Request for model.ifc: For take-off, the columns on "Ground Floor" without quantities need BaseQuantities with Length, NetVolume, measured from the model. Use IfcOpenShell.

First a look at what the model holds.

```python
import ifcopenshell
import ifcopenshell.util.element
import ifcopenshell.util.unit

model = ifcopenshell.open("model.ifc")
print(model.schema)
for unit_type in ("LENGTHUNIT", "AREAUNIT", "VOLUMEUNIT"):
    print(unit_type, ifcopenshell.util.unit.calculate_unit_scale(model, unit_type))
storey = next(s for s in model.by_type("IfcBuildingStorey") if s.Name == "Ground Floor")
columns = [e for e in ifcopenshell.util.element.get_decomposition(storey) if e.is_a("IfcColumn")]
for e in sorted(columns, key=lambda e: e.id()):
    print(e.id(), e.is_a(), e.Name, list(ifcopenshell.util.element.get_psets(e, qtos_only=True)), sep=" | ")
```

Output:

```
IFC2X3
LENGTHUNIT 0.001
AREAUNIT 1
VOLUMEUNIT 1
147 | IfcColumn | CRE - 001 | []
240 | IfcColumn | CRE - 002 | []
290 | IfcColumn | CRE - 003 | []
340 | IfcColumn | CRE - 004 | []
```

```python
import ifcopenshell
import ifcopenshell.api.pset
import ifcopenshell.geom
import ifcopenshell.util.element
import ifcopenshell.util.shape
import ifcopenshell.util.unit

model = ifcopenshell.open("model.ifc")
unit_scale = ifcopenshell.util.unit.calculate_unit_scale(model)
volume_scale = ifcopenshell.util.unit.calculate_unit_scale(model, "VOLUMEUNIT")
settings = ifcopenshell.geom.settings()

storey = next(s for s in model.by_type("IfcBuildingStorey") if s.Name == "Ground Floor")
columns = [e for e in ifcopenshell.util.element.get_decomposition(storey) if e.is_a("IfcColumn")]

for e in sorted(columns, key=lambda e: e.id()):
    if ifcopenshell.util.element.get_psets(e, qtos_only=True, should_inherit=False):
        continue
    # Geometry comes back in metres, in the element's own axes.
    shape = ifcopenshell.geom.create_shape(settings, e)
    values = {
        "Length": ifcopenshell.util.shape.get_z(shape.geometry) / unit_scale,
        "NetVolume": ifcopenshell.util.shape.get_volume(shape.geometry) / volume_scale,
    }
    qto = ifcopenshell.api.pset.add_qto(model, product=e, name="BaseQuantities")
    ifcopenshell.api.pset.edit_qto(model, qto=qto, properties=values)
    print(e.id(), {k: round(v, 3) for k, v in values.items()})

model.write("model_v2.ifc")
```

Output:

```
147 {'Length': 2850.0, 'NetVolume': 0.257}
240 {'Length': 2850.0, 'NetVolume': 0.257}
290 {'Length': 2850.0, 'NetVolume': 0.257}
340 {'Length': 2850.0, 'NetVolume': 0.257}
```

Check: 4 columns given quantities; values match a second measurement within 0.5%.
